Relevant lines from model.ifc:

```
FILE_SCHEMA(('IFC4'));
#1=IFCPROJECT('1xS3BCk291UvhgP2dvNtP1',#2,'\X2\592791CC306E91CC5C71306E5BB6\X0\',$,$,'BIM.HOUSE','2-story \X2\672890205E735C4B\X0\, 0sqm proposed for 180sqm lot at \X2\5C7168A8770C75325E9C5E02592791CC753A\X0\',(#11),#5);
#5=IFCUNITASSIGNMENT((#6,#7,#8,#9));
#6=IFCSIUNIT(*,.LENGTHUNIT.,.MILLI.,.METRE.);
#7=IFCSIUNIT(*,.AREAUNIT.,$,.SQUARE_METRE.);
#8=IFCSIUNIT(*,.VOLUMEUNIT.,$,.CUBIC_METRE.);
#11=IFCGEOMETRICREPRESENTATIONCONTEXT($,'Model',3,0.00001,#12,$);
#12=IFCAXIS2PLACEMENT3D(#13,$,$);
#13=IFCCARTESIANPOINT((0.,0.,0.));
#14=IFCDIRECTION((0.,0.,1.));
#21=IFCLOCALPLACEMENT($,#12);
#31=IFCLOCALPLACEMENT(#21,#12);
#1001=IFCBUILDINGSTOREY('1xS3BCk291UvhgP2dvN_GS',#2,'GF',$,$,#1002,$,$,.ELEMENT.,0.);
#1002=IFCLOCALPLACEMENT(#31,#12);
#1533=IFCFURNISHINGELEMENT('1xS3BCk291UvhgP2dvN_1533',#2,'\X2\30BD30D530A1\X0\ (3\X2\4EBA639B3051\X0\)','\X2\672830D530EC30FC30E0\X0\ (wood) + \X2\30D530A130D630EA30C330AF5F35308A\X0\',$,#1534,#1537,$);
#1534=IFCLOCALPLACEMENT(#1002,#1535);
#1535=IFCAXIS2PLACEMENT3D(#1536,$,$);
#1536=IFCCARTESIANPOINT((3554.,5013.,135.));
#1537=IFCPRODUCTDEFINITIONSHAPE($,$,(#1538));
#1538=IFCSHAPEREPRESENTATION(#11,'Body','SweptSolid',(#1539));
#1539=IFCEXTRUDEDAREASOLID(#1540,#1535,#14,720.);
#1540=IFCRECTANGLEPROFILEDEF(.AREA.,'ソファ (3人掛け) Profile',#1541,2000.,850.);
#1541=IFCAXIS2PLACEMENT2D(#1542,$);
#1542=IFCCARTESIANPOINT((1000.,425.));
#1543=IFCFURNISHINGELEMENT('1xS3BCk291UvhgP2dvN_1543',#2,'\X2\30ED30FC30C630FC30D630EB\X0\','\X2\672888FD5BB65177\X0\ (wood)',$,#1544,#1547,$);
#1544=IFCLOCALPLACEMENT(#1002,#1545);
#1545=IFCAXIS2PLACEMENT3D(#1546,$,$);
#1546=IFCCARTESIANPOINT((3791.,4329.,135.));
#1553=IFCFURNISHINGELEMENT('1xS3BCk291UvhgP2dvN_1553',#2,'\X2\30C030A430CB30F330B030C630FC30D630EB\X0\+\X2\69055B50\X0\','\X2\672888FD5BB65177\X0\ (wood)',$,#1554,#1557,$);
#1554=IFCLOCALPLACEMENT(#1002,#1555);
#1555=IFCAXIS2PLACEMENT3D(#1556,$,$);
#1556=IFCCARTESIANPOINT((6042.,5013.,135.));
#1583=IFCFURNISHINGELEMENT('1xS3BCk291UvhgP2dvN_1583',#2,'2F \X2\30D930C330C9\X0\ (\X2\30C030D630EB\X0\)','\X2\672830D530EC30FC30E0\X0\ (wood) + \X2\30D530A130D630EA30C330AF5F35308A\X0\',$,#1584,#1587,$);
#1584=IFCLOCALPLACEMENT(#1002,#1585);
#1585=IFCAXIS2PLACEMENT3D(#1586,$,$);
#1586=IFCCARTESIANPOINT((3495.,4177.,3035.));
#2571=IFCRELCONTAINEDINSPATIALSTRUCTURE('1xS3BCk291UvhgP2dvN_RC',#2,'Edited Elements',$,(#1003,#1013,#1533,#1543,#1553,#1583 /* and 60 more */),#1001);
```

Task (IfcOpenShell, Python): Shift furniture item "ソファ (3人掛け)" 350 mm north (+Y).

```python
import ifcopenshell
import ifcopenshell.api.geometry
import ifcopenshell.util.placement
import ifcopenshell.util.unit

model = ifcopenshell.open("model.ifc")
unit_scale = ifcopenshell.util.unit.calculate_unit_scale(model)

item = model.by_guid("1xS3BCk291UvhgP2dvN_1533")
matrix = ifcopenshell.util.placement.get_local_placement(item.ObjectPlacement)
matrix[1, 3] += 0.35 / unit_scale
ifcopenshell.api.geometry.edit_object_placement(model, product=item, matrix=matrix, is_si=False)

print(ifcopenshell.util.placement.get_local_placement(item.ObjectPlacement).round(3) + 0.0)

model.write("model_rev.ifc")
```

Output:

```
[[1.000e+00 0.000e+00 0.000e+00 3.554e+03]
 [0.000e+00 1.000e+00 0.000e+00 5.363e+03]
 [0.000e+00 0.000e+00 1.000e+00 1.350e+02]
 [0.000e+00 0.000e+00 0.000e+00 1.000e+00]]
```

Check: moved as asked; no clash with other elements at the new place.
